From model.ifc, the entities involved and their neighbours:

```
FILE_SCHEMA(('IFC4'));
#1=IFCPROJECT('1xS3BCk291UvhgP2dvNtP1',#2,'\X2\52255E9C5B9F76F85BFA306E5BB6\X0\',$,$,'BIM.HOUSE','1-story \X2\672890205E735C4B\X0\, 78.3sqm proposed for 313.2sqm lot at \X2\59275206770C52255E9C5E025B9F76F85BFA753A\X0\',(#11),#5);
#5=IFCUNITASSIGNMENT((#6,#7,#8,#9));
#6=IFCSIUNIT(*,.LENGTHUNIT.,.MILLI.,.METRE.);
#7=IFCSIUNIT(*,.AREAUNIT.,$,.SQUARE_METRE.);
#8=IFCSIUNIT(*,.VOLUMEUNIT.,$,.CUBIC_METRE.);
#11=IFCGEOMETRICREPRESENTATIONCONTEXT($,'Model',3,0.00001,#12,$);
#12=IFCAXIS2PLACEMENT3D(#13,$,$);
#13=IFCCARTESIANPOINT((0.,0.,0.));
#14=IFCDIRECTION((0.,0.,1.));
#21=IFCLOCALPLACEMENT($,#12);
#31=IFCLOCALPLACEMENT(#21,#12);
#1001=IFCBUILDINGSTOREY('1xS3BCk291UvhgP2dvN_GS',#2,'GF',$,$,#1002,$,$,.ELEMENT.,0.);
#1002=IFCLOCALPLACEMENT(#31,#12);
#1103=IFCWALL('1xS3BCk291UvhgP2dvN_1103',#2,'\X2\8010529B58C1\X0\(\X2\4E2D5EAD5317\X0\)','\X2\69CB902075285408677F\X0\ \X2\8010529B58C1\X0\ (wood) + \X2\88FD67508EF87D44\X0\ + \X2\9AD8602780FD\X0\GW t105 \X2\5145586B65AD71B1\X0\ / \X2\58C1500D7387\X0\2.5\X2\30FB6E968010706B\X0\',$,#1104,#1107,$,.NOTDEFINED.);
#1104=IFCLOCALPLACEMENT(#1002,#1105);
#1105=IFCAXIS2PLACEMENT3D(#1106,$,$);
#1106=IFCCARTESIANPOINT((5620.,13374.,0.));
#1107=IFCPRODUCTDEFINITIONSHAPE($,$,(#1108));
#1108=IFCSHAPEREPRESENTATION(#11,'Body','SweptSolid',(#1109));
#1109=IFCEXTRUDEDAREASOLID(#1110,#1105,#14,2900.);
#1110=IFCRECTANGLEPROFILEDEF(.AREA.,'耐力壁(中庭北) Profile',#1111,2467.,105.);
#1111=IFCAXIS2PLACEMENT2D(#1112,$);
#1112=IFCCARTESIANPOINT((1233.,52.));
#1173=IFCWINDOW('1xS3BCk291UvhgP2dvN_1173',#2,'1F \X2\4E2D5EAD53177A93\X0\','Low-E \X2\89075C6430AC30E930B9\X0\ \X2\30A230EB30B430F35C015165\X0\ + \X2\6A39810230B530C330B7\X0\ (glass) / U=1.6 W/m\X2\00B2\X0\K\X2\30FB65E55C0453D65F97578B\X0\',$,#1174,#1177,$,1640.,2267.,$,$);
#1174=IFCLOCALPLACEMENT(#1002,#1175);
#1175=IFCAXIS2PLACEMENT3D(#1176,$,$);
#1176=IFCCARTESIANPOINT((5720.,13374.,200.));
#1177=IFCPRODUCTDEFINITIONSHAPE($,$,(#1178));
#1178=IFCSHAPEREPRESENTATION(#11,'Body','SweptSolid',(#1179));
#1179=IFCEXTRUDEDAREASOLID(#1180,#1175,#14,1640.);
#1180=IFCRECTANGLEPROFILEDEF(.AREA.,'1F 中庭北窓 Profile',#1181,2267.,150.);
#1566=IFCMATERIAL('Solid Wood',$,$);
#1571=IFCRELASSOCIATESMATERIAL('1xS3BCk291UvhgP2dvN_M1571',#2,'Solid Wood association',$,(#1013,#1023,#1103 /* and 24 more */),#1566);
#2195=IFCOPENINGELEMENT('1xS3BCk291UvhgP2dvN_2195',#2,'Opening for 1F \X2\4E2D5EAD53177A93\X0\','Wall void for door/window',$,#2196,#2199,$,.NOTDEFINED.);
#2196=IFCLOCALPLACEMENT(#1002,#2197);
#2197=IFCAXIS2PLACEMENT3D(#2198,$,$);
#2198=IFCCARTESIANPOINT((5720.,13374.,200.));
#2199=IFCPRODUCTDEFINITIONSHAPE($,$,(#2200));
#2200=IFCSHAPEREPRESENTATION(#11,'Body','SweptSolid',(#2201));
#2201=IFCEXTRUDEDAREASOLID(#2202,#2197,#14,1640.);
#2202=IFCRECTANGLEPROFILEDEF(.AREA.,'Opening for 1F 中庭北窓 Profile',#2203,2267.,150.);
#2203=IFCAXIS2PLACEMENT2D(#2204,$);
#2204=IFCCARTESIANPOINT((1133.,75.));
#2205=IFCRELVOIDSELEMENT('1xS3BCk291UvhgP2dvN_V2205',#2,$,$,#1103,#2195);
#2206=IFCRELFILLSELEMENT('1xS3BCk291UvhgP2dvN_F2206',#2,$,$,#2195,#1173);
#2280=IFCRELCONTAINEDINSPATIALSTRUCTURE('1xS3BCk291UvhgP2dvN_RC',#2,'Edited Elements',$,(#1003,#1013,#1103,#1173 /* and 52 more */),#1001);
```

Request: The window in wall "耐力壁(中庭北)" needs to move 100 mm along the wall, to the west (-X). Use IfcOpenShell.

```python
import ifcopenshell
import ifcopenshell.api.geometry
import ifcopenshell.util.placement

model = ifcopenshell.open("model.ifc")

window = model.by_id(1173)
opening = window.FillsVoids[0].RelatingOpeningElement
wall = opening.VoidsElements[0].RelatingBuildingElement

wall_matrix = ifcopenshell.util.placement.get_local_placement(wall.ObjectPlacement)
shift = wall_matrix[:3, 0] * -100.0
before = ifcopenshell.util.placement.get_local_placement(window.ObjectPlacement)[:3, 3].copy()

# The window is not placed relative to its opening, so move both.
for product in (opening, window):
    matrix = ifcopenshell.util.placement.get_local_placement(product.ObjectPlacement)
    matrix[:3, 3] += shift
    ifcopenshell.api.geometry.edit_object_placement(model, product=product, matrix=matrix, is_si=False)

after = ifcopenshell.util.placement.get_local_placement(window.ObjectPlacement)[:3, 3]
print("window moved by", (after - before).round(3) + 0.0)

model.write("model_rev.ifc")
```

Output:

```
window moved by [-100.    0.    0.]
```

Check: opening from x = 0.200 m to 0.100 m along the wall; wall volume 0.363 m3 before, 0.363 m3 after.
